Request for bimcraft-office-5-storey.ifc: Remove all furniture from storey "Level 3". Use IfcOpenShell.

First a look at what the model holds.

```python
import ifcopenshell
import ifcopenshell.util.element

model = ifcopenshell.open("bimcraft-office-5-storey.ifc")
print(model.schema)
storey = next(s for s in model.by_type("IfcBuildingStorey") if s.Name == "Level 3")
furniture = [e for e in ifcopenshell.util.element.get_decomposition(storey) if e.is_a("IfcFurnishingElement")]
seen = {}
for e in furniture:
    element_type = ifcopenshell.util.element.get_type(e)
    name = element_type.Name if element_type not in (None, e) else None
    seen[name] = seen.get(name, 0) + 1
for name, count in sorted(seen.items(), key=str):
    print(count, "x", name)
```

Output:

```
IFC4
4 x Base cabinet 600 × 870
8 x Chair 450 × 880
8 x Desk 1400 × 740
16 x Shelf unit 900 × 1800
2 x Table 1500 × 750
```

```python
import ifcopenshell
import ifcopenshell.api.root
import ifcopenshell.util.element

model = ifcopenshell.open("bimcraft-office-5-storey.ifc")

storey = next(s for s in model.by_type("IfcBuildingStorey") if s.Name == "Level 3")
furniture = [e for e in ifcopenshell.util.element.get_decomposition(storey) if e.is_a("IfcFurnishingElement")]

for e in furniture:
    ifcopenshell.api.root.remove_product(model, product=e)
print(len(furniture), "removed")

model.write("bimcraft-office-5-storey_rev.ifc")
```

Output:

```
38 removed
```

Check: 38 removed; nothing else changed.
